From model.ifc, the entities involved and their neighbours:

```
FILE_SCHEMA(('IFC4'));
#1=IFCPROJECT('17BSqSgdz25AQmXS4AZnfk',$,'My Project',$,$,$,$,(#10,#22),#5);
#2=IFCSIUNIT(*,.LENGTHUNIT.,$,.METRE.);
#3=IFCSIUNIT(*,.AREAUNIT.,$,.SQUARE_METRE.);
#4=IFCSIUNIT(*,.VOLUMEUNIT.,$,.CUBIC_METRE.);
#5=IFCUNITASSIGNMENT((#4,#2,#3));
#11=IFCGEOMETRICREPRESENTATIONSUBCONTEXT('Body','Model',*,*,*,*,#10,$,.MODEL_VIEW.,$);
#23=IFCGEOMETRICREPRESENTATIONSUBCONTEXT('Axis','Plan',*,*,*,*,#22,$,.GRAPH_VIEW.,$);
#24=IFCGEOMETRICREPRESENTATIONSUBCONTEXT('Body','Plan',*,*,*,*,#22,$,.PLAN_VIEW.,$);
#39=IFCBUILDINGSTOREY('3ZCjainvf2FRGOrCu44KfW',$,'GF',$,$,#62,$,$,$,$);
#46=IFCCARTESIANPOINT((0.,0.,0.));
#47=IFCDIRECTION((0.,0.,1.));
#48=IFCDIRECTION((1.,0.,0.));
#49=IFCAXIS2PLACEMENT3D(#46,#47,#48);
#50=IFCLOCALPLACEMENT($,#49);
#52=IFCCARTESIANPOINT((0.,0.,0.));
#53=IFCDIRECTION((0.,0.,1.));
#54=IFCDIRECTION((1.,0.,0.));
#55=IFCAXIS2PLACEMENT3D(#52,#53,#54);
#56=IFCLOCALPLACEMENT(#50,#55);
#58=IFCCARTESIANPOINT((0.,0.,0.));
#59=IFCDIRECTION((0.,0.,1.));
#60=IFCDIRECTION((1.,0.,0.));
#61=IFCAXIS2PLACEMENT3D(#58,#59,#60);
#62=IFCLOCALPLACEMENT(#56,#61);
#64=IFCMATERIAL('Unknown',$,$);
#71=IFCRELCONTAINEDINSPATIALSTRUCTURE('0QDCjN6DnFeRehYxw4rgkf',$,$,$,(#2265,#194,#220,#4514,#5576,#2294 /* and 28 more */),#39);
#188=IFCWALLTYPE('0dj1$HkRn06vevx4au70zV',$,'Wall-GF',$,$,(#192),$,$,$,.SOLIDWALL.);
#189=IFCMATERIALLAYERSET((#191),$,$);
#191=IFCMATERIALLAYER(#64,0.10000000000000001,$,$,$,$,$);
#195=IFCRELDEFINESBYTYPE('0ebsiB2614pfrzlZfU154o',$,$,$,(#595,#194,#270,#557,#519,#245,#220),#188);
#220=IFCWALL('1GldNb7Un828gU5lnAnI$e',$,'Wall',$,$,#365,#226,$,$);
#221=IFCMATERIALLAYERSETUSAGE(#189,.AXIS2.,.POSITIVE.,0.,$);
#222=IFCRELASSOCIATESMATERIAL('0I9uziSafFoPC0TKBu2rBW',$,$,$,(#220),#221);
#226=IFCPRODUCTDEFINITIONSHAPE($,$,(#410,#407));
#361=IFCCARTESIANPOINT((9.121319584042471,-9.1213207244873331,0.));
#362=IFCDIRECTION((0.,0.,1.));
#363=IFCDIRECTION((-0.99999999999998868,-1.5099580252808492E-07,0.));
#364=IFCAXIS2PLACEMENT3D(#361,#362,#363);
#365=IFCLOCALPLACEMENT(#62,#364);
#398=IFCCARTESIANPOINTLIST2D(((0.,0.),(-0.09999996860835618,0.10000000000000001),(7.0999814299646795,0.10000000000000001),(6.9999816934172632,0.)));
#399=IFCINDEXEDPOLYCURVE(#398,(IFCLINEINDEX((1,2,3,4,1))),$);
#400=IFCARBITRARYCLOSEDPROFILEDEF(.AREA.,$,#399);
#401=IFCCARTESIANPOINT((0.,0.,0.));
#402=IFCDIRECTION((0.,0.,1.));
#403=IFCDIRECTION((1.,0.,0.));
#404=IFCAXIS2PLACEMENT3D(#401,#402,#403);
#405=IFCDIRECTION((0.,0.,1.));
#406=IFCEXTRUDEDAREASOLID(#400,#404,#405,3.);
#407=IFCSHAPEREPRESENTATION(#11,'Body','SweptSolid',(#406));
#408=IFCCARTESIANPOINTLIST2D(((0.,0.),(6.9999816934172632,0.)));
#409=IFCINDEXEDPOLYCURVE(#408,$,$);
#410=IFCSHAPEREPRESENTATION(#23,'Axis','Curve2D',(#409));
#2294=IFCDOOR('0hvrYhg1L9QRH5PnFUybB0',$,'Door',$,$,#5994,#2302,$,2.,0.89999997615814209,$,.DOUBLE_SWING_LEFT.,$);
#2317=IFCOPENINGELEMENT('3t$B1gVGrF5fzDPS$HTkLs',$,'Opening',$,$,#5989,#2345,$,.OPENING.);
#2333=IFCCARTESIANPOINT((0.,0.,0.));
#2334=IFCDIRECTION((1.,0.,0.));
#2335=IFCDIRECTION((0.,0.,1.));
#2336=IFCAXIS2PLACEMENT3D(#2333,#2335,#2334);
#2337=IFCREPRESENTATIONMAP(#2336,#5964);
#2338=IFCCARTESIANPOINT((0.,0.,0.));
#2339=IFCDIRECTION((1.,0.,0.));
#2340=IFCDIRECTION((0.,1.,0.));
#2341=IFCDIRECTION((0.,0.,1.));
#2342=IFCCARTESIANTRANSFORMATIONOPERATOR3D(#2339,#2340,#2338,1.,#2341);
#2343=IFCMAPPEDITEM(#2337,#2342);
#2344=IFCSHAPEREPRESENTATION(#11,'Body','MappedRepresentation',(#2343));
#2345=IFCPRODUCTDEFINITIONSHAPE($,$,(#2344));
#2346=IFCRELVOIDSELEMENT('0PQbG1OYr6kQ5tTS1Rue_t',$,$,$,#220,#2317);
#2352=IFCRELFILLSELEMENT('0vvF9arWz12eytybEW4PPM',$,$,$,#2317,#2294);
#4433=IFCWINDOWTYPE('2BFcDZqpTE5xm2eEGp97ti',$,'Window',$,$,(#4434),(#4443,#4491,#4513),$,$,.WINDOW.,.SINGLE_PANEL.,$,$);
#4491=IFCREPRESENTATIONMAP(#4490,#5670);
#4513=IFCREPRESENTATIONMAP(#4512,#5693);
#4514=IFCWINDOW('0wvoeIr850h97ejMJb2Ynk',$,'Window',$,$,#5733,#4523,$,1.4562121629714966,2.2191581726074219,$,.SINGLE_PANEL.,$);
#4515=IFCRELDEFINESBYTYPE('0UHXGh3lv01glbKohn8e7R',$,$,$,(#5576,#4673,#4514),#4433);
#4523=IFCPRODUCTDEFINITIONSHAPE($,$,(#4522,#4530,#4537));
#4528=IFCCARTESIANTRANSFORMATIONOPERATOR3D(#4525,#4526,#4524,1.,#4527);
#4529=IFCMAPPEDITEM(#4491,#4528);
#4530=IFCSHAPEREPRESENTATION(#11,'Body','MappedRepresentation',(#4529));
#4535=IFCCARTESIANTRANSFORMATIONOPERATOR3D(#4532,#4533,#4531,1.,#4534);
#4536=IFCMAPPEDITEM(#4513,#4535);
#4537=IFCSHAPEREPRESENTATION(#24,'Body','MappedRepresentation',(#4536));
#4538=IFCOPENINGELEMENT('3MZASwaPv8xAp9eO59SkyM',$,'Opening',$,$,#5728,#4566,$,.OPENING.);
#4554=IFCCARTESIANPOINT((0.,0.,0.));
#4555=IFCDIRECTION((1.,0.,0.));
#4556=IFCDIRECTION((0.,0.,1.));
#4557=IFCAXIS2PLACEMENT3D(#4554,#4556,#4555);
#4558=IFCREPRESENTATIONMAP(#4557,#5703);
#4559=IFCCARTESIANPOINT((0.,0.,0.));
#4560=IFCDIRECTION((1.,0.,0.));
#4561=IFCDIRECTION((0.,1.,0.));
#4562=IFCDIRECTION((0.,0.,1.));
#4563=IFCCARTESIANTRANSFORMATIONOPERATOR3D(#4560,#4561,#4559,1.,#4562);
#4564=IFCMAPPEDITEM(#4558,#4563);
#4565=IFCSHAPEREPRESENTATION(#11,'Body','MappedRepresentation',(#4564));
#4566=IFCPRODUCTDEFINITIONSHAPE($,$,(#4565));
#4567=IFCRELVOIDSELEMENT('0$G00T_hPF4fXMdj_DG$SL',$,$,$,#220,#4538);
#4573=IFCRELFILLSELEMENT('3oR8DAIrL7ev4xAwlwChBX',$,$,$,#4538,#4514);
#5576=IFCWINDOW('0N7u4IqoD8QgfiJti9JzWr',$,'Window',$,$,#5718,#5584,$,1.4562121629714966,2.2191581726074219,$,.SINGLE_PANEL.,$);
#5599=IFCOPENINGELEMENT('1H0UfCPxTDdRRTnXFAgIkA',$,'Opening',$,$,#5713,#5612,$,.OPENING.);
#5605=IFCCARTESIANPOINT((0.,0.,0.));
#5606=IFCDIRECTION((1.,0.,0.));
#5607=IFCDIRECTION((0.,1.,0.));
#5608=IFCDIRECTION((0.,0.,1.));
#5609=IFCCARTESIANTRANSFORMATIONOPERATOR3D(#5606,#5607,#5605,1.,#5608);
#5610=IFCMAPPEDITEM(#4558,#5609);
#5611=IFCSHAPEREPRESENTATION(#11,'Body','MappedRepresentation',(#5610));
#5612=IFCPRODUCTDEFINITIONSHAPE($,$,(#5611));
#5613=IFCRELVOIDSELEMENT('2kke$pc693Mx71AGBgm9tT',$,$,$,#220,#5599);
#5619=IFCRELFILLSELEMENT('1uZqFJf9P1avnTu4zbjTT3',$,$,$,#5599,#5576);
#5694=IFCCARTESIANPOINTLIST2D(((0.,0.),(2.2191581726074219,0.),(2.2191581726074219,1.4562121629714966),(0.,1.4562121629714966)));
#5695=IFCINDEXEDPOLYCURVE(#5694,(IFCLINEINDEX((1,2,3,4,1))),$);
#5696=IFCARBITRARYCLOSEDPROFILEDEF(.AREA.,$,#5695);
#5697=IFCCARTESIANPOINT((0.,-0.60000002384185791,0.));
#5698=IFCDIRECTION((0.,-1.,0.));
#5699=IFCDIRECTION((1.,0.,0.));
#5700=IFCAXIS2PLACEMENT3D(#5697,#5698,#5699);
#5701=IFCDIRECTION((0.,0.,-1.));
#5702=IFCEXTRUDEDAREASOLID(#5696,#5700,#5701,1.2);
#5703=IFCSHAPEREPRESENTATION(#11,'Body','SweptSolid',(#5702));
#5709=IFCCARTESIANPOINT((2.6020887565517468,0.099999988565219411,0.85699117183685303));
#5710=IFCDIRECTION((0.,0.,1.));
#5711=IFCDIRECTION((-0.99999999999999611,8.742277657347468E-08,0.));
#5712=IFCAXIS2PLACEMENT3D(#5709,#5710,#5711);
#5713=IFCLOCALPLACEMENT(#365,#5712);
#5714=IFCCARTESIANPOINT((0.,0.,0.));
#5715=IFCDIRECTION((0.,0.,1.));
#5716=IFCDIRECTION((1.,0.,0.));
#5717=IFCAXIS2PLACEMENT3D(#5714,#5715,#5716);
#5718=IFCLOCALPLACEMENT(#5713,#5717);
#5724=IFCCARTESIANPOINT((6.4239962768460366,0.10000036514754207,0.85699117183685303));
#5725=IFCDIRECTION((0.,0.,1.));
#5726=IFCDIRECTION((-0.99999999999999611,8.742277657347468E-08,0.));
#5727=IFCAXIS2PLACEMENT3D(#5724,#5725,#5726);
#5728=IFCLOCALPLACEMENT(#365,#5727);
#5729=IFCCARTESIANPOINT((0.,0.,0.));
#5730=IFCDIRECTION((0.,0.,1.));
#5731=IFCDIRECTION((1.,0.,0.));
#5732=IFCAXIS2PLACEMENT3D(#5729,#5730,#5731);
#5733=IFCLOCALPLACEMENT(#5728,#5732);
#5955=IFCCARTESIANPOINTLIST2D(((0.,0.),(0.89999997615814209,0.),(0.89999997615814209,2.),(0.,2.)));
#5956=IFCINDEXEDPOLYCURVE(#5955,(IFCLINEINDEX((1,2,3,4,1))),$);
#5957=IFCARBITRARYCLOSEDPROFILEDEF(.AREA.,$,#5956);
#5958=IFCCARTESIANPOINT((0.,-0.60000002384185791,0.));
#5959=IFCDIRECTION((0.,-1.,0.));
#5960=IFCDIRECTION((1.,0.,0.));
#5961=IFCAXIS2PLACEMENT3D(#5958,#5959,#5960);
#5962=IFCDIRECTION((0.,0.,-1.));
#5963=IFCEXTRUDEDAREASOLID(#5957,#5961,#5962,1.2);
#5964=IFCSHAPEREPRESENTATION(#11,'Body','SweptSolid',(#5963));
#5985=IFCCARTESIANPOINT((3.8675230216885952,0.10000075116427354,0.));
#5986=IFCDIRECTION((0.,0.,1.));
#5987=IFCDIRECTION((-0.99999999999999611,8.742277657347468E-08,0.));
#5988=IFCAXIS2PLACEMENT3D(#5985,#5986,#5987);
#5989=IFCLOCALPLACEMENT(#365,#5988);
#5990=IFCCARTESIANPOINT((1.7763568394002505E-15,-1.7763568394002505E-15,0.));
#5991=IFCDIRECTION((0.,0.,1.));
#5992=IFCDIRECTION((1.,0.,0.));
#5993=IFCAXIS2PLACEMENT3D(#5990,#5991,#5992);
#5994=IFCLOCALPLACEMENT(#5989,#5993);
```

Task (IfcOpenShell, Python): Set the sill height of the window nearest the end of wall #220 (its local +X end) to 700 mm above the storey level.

```python
import numpy as np
import ifcopenshell
import ifcopenshell.api.geometry
import ifcopenshell.geom
import ifcopenshell.util.element
import ifcopenshell.util.placement
import ifcopenshell.util.shape
import ifcopenshell.util.unit

model = ifcopenshell.open("model.ifc")
unit_scale = ifcopenshell.util.unit.calculate_unit_scale(model)

window = model.by_guid("0wvoeIr850h97ejMJb2Ynk")
opening = window.FillsVoids[0].RelatingOpeningElement
storey = ifcopenshell.util.element.get_container(window, ifc_class="IfcBuildingStorey")
level = ifcopenshell.util.placement.get_local_placement(storey.ObjectPlacement)[2, 3]

# The opening's origin need not be at the sill, so measure its lowest point.
shape = ifcopenshell.geom.create_shape(ifcopenshell.geom.settings(), opening)
bottom = ifcopenshell.util.shape.get_shape_bottom_elevation(shape, shape.geometry) / unit_scale
dz = level + 0.7 / unit_scale - bottom

shift = np.array([0.0, 0.0, dz])
# The window is placed relative to its opening, so it follows when the opening moves.
matrix = ifcopenshell.util.placement.get_local_placement(opening.ObjectPlacement)
matrix[:3, 3] += shift
ifcopenshell.api.geometry.edit_object_placement(
    model, product=opening, matrix=matrix, is_si=False, should_transform_children=True
)

print(f"moved by {dz * unit_scale:+.3f} m")

model.write("model_v2.ifc")
```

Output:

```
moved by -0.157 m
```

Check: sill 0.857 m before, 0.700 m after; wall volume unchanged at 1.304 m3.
